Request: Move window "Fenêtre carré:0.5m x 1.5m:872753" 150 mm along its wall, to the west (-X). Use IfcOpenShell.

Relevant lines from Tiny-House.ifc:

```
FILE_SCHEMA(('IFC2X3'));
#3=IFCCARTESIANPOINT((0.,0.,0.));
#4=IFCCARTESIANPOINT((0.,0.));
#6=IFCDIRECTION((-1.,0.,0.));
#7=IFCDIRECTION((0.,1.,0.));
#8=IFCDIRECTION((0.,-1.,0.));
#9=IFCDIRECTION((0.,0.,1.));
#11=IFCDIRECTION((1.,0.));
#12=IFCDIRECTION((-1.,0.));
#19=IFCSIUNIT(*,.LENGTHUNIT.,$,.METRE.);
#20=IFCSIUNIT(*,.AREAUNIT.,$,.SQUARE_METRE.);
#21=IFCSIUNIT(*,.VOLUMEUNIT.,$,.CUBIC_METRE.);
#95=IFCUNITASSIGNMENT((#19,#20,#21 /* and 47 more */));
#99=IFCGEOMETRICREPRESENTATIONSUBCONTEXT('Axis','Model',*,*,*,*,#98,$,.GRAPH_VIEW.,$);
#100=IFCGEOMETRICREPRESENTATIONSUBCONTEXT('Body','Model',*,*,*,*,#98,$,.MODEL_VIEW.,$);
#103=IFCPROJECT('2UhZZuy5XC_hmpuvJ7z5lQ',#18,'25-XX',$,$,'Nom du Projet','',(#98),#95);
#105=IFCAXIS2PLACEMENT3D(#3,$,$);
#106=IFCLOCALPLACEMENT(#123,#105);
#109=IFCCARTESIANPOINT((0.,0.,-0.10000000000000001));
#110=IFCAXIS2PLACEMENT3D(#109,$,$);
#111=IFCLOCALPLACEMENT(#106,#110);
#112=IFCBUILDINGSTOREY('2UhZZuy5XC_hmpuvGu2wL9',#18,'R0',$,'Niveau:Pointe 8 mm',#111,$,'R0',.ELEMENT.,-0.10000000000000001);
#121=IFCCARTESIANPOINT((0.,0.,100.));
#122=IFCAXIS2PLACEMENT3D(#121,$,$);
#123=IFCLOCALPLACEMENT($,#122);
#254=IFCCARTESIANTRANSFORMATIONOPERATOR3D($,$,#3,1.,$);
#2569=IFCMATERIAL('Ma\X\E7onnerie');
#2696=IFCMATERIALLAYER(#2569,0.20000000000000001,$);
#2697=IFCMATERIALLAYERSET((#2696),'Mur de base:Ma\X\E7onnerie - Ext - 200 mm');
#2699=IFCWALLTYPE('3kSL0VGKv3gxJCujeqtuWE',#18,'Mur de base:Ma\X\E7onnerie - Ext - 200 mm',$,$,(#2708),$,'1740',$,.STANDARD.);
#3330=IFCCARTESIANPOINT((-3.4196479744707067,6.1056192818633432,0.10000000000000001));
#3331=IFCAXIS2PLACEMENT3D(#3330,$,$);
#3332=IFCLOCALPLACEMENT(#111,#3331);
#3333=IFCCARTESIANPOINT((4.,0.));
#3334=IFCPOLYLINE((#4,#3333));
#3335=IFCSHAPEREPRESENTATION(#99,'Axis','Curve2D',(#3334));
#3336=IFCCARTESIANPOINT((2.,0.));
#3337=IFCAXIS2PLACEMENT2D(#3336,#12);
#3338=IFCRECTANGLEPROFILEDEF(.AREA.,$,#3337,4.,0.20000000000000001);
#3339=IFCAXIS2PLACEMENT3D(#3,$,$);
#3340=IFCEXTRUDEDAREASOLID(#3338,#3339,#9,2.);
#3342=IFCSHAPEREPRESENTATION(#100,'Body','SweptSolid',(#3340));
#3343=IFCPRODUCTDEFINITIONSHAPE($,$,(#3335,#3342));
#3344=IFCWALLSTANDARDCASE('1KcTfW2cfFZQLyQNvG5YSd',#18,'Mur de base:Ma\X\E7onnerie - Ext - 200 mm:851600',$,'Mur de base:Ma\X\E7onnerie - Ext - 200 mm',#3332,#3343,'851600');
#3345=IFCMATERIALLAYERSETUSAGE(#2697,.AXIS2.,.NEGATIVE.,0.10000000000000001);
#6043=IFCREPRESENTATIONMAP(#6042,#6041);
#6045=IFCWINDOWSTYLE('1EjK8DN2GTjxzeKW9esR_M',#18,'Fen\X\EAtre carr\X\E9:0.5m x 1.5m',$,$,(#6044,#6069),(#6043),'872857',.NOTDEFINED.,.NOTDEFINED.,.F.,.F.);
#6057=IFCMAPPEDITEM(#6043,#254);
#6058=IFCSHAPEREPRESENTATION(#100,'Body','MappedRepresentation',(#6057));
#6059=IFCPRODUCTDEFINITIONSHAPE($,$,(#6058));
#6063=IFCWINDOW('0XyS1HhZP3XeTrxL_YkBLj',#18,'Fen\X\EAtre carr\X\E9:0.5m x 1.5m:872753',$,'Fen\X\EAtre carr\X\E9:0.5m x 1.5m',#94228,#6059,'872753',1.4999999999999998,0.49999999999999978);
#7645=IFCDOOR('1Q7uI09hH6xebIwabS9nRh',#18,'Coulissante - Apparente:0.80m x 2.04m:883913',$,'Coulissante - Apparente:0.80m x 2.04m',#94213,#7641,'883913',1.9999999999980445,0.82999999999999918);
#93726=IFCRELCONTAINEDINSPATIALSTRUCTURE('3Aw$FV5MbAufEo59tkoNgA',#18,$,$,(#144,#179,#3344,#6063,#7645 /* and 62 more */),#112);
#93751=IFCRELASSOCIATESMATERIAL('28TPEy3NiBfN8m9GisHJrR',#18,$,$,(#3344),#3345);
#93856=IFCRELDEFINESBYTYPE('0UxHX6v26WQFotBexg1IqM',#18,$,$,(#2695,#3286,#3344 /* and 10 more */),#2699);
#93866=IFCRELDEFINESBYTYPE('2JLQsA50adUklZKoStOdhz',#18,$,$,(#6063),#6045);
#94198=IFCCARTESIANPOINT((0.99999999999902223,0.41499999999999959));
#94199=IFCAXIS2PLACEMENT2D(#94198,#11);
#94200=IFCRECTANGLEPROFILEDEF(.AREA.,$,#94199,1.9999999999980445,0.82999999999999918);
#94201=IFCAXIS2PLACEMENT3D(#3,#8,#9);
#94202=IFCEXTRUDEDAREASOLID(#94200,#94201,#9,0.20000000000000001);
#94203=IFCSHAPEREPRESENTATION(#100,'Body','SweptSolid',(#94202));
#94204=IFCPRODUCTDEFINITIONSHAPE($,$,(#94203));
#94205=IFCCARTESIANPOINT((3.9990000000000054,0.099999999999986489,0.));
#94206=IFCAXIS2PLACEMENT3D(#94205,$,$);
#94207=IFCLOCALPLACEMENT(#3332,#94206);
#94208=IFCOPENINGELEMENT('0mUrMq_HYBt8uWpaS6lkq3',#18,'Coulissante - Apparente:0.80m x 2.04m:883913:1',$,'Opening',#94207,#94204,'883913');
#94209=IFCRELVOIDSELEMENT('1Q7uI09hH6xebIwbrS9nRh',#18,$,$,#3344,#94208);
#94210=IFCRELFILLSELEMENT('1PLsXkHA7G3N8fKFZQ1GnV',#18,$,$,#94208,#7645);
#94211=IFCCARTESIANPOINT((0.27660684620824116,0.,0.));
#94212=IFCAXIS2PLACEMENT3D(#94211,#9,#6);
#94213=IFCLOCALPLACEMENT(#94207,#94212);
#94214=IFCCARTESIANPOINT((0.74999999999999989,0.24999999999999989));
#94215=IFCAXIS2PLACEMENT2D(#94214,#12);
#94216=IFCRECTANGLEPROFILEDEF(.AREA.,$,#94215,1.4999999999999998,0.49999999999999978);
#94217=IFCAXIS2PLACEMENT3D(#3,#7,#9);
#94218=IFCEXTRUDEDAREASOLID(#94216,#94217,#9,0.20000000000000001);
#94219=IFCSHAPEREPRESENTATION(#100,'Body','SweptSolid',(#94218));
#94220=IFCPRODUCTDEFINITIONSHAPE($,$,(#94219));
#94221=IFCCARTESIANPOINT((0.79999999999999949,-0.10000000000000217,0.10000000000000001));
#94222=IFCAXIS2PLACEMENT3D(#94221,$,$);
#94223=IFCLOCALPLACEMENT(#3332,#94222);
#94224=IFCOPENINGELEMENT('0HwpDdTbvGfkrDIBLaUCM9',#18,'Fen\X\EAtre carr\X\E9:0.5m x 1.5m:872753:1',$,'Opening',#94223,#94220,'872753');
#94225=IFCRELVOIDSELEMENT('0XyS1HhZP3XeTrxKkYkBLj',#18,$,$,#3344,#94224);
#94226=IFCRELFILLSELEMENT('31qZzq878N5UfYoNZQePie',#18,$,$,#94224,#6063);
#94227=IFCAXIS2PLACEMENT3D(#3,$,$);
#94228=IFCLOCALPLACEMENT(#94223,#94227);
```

```python
import ifcopenshell
import ifcopenshell.api.geometry
import ifcopenshell.util.placement
import ifcopenshell.util.unit

model = ifcopenshell.open("Tiny-House.ifc")
unit_scale = ifcopenshell.util.unit.calculate_unit_scale(model)

window = model.by_id(6063)
opening = window.FillsVoids[0].RelatingOpeningElement
wall = opening.VoidsElements[0].RelatingBuildingElement

wall_matrix = ifcopenshell.util.placement.get_local_placement(wall.ObjectPlacement)
shift = wall_matrix[:3, 0] * -0.15 / unit_scale
before = ifcopenshell.util.placement.get_local_placement(window.ObjectPlacement)[:3, 3].copy()

# The window is placed relative to its opening, so it follows when the opening moves.
matrix = ifcopenshell.util.placement.get_local_placement(opening.ObjectPlacement)
matrix[:3, 3] += shift
ifcopenshell.api.geometry.edit_object_placement(
    model, product=opening, matrix=matrix, is_si=False, should_transform_children=True
)

after = ifcopenshell.util.placement.get_local_placement(window.ObjectPlacement)[:3, 3]
print("window moved by", (after - before).round(3) + 0.0)

model.write("Tiny-House_rev.ifc")
```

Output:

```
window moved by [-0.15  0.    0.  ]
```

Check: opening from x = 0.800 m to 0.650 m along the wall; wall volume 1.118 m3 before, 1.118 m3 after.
